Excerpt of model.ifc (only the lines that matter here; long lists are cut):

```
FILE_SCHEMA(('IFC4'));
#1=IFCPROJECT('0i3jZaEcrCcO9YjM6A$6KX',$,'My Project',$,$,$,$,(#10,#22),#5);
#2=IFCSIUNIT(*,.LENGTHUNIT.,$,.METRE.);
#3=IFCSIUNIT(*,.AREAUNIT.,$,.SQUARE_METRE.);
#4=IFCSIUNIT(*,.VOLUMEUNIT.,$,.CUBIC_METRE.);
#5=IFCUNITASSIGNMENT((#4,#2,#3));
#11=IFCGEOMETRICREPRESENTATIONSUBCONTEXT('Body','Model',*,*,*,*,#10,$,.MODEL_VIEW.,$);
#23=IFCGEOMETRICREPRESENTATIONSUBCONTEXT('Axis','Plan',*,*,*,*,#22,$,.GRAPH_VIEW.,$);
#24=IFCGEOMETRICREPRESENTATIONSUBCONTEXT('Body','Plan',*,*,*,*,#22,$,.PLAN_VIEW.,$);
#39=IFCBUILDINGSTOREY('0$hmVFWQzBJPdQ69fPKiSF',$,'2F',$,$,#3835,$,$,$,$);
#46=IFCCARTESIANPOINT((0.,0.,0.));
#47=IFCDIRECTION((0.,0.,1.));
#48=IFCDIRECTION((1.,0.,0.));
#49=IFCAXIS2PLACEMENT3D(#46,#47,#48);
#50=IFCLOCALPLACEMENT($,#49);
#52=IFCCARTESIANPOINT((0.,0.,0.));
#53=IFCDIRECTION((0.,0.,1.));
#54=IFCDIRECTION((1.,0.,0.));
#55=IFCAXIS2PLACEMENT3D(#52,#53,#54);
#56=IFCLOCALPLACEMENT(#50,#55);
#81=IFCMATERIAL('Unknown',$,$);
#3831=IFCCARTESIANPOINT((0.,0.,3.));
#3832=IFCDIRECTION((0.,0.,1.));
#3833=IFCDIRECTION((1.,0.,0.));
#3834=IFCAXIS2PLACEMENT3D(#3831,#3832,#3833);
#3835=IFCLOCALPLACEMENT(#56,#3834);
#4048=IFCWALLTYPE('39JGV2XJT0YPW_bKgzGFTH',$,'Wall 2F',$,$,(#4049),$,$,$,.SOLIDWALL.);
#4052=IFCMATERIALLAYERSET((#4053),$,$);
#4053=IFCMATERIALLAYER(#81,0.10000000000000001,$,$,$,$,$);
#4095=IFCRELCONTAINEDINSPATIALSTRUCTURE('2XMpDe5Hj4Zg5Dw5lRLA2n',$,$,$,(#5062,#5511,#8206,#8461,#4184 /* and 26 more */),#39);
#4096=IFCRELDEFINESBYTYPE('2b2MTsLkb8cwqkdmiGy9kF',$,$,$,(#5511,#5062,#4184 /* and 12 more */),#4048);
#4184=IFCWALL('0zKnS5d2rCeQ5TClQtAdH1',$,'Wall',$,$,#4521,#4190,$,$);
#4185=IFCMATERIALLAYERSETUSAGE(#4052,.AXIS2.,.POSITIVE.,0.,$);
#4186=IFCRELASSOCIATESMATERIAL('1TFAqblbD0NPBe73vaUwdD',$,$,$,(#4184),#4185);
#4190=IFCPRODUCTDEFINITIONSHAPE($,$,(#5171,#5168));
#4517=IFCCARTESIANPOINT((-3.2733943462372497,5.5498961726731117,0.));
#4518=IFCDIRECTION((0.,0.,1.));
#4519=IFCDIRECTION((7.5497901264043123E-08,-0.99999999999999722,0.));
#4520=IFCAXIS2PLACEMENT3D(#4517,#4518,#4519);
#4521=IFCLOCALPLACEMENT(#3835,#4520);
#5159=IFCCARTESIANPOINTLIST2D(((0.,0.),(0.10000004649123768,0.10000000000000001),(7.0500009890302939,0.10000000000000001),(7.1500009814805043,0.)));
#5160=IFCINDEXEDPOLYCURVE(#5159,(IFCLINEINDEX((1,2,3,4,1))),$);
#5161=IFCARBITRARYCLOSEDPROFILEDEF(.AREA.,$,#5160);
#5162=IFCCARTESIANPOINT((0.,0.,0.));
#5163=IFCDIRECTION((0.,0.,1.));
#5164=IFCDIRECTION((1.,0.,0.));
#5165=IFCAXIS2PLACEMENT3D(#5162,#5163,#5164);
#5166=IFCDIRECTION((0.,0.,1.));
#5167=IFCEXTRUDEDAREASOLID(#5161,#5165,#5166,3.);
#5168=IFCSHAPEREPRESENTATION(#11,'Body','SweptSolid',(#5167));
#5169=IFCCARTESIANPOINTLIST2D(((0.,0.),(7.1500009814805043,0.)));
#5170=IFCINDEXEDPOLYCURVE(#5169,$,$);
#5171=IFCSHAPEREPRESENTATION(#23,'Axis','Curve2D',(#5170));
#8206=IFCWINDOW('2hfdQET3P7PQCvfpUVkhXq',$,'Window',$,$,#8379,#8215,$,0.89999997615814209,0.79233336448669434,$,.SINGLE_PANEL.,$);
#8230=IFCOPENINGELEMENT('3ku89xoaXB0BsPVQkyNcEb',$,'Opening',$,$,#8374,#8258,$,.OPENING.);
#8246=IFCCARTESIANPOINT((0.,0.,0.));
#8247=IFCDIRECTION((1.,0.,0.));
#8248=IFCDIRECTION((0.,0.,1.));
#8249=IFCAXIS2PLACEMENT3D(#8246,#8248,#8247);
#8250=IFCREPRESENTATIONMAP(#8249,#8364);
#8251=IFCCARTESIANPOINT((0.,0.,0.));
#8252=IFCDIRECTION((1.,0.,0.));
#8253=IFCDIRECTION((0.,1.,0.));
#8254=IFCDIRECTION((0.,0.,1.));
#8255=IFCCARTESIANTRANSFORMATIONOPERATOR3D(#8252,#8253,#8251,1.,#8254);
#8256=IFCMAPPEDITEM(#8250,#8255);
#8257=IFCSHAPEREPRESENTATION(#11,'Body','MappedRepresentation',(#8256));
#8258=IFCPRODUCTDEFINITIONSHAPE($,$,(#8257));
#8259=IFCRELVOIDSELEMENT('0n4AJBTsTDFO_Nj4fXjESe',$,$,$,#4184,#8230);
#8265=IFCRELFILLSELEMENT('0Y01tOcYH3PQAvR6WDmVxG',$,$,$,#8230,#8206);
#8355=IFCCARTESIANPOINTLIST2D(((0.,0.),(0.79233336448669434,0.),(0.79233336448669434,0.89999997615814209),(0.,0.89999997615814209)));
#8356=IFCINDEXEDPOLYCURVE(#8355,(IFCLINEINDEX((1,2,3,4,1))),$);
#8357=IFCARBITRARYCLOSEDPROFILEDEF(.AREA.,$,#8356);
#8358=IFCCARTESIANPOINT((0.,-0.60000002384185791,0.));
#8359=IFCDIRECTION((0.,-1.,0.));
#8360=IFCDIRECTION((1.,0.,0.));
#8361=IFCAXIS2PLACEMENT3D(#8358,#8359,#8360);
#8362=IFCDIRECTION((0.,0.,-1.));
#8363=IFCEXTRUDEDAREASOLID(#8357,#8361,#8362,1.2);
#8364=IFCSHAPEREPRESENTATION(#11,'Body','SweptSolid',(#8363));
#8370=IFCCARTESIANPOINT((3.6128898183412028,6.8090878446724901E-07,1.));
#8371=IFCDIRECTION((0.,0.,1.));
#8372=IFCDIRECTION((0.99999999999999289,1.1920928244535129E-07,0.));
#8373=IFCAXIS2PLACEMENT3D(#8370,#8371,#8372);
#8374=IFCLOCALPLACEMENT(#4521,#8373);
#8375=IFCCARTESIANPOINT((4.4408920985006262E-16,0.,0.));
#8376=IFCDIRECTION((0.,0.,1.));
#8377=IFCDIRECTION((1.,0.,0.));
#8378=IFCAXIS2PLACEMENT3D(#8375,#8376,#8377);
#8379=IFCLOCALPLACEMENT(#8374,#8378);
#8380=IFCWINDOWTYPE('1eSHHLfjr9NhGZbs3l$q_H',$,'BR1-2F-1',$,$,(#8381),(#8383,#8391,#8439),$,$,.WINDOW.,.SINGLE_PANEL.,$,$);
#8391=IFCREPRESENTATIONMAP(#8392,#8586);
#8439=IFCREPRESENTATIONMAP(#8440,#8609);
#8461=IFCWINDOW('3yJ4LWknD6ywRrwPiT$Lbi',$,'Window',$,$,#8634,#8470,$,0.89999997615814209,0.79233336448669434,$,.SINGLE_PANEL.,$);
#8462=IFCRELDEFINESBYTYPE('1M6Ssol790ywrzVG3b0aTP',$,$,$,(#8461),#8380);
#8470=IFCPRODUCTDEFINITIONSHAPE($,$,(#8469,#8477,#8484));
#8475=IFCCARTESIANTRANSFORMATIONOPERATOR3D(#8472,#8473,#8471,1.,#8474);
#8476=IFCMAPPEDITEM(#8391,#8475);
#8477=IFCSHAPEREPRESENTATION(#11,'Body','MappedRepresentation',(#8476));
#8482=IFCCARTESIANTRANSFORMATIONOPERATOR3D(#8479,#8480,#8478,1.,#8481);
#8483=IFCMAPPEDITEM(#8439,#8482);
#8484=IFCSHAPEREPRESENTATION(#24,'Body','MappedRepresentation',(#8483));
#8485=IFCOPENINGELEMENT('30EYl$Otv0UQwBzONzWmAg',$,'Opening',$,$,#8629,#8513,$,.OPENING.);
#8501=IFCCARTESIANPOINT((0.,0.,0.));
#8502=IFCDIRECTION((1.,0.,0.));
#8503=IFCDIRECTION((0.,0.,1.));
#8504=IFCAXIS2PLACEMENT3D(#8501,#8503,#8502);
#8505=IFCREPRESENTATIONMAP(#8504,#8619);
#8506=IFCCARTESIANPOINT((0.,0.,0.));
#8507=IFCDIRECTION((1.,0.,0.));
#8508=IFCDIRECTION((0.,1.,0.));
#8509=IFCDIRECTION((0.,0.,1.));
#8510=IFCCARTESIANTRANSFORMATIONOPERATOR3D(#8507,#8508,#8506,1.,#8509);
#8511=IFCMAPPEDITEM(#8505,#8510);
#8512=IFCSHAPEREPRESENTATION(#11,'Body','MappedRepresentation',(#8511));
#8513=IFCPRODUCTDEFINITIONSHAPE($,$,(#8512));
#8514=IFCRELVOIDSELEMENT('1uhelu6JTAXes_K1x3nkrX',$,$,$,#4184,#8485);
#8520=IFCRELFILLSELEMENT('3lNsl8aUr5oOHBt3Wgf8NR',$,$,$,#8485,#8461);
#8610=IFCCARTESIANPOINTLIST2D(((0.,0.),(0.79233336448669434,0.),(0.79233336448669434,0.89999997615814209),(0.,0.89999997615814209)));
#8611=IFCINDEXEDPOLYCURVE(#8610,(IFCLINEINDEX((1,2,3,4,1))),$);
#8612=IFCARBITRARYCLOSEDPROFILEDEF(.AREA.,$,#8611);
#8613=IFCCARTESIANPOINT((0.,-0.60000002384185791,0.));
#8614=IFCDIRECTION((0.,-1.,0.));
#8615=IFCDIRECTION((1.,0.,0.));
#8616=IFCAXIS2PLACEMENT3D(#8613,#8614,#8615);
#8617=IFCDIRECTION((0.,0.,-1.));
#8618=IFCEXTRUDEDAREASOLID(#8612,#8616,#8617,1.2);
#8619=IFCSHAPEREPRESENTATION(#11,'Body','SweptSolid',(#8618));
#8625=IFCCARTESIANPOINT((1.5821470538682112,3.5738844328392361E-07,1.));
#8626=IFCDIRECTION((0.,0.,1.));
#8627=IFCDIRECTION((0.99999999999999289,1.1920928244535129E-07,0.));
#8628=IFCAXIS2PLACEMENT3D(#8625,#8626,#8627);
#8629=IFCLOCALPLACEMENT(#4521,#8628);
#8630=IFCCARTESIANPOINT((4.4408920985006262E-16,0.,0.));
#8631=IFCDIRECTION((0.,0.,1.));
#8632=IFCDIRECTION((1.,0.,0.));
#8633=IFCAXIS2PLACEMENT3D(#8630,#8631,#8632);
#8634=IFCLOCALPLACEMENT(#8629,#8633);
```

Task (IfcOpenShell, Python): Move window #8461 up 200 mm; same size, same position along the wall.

```python
import numpy as np
import ifcopenshell
import ifcopenshell.api.geometry
import ifcopenshell.util.placement
import ifcopenshell.util.unit

model = ifcopenshell.open("model.ifc")
unit_scale = ifcopenshell.util.unit.calculate_unit_scale(model)

window = model.by_guid("3yJ4LWknD6ywRrwPiT$Lbi")
opening = window.FillsVoids[0].RelatingOpeningElement
dz = 0.2 / unit_scale

shift = np.array([0.0, 0.0, dz])
# The window is placed relative to its opening, so it follows when the opening moves.
matrix = ifcopenshell.util.placement.get_local_placement(opening.ObjectPlacement)
matrix[:3, 3] += shift
ifcopenshell.api.geometry.edit_object_placement(
    model, product=opening, matrix=matrix, is_si=False, should_transform_children=True
)

print(f"moved by {dz * unit_scale:+.3f} m")

model.write("model_edited.ifc")
```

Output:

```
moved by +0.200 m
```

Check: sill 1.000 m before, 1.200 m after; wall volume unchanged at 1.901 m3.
